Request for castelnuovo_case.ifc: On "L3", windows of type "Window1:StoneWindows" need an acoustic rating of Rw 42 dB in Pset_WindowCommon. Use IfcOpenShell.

First a look at what the model holds.

```python
import ifcopenshell
import ifcopenshell.util.element

model = ifcopenshell.open("castelnuovo_case.ifc")
print(model.schema)
storey = next(s for s in model.by_type("IfcBuildingStorey") if s.Name == "L3")
windows = [e for e in ifcopenshell.util.element.get_decomposition(storey) if e.is_a("IfcWindow")]
seen = {}
for e in windows:
    element_type = ifcopenshell.util.element.get_type(e)
    key = (element_type.Name if element_type != e and element_type else None, ifcopenshell.util.element.get_pset(e, "Pset_WindowCommon", "AcousticRating"))
    seen[key] = seen.get(key, 0) + 1
for (name, value), count in sorted(seen.items(), key=str):
    print(count, "x", name, "|", value)
```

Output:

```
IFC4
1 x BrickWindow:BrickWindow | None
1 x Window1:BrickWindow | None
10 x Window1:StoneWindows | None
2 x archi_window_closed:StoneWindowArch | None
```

```python
import ifcopenshell
import ifcopenshell.api.pset
import ifcopenshell.util.element

model = ifcopenshell.open("castelnuovo_case.ifc")

storey = next(s for s in model.by_type("IfcBuildingStorey") if s.Name == "L3")
windows = [e for e in ifcopenshell.util.element.get_decomposition(storey) if e.is_a("IfcWindow")]

count = 0
for e in windows:
    element_type = ifcopenshell.util.element.get_type(e)
    if element_type in (None, e) or element_type.Name != "Window1:StoneWindows":
        continue
    # add_pset returns the element's existing set when there is one.
    pset = ifcopenshell.api.pset.add_pset(model, product=e, name="Pset_WindowCommon")
    ifcopenshell.api.pset.edit_pset(model, pset=pset, properties={"AcousticRating": "Rw 42 dB"})
    count += 1

print(count, "windows updated")

model.write("castelnuovo_case-out.ifc")
```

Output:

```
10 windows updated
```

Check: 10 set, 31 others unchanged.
